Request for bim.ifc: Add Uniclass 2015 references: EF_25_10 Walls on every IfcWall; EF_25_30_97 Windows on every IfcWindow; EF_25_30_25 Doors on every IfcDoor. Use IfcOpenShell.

First a look at what the model holds.

```python
import ifcopenshell

model = ifcopenshell.open("bim.ifc")
print(model.schema)
print("classifications:", [c.Name for c in model.by_type("IfcClassification")])
for ifc_class in ("IfcDoor", "IfcRoof", "IfcStair", "IfcWall", "IfcWindow"):
    print(ifc_class, len(model.by_type(ifc_class)))
```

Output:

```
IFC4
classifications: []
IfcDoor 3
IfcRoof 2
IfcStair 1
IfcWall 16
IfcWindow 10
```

```python
import ifcopenshell
import ifcopenshell.api.classification

model = ifcopenshell.open("bim.ifc")

system = ifcopenshell.api.classification.add_classification(model, classification="Uniclass 2015")

codes = {
    "IfcWall": ("EF_25_10", "Walls"),
    "IfcWindow": ("EF_25_30_97", "Windows"),
    "IfcDoor": ("EF_25_30_25", "Doors"),
}
for ifc_class, (code, name) in codes.items():
    products = model.by_type(ifc_class)
    ifcopenshell.api.classification.add_reference(
        model, products=products, classification=system, identification=code, name=name
    )
    print(code, len(products))

model.write("bim_rev.ifc")
```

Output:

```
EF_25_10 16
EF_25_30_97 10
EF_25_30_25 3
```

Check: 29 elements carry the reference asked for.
